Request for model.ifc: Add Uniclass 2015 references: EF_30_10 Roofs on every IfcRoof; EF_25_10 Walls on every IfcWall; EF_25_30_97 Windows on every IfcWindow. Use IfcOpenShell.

First a look at what the model holds.

```python
import ifcopenshell

model = ifcopenshell.open("model.ifc")
print(model.schema)
print("classifications:", [c.Name for c in model.by_type("IfcClassification")])
for ifc_class in ("IfcDoor", "IfcRoof", "IfcStair", "IfcWall", "IfcWindow"):
    print(ifc_class, len(model.by_type(ifc_class)))
```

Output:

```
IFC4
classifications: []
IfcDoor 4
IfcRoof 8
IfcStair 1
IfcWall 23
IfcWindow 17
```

```python
import ifcopenshell
import ifcopenshell.api.classification

model = ifcopenshell.open("model.ifc")

system = ifcopenshell.api.classification.add_classification(model, classification="Uniclass 2015")

codes = {
    "IfcRoof": ("EF_30_10", "Roofs"),
    "IfcWall": ("EF_25_10", "Walls"),
    "IfcWindow": ("EF_25_30_97", "Windows"),
}
for ifc_class, (code, name) in codes.items():
    products = model.by_type(ifc_class)
    ifcopenshell.api.classification.add_reference(
        model, products=products, classification=system, identification=code, name=name
    )
    print(code, len(products))

model.write("model_rev.ifc")
```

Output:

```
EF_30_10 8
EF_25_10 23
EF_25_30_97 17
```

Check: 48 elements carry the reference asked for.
